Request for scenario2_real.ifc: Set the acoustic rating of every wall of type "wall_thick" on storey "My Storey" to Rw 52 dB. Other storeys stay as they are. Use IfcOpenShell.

First a look at what the model holds.

```python
import ifcopenshell
import ifcopenshell.util.element

model = ifcopenshell.open("scenario2_real.ifc")
print(model.schema)
storey = next(s for s in model.by_type("IfcBuildingStorey") if s.Name == "My Storey")
walls = [e for e in ifcopenshell.util.element.get_decomposition(storey) if e.is_a("IfcWall")]
seen = {}
for e in walls:
    element_type = ifcopenshell.util.element.get_type(e)
    key = (element_type.Name if element_type != e and element_type else None, ifcopenshell.util.element.get_pset(e, "Pset_WallCommon", "AcousticRating"))
    seen[key] = seen.get(key, 0) + 1
for (name, value), count in sorted(seen.items(), key=str):
    print(count, "x", name, "|", value)
```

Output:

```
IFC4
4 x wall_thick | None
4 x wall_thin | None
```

```python
import ifcopenshell
import ifcopenshell.api.pset
import ifcopenshell.util.element

model = ifcopenshell.open("scenario2_real.ifc")

storey = next(s for s in model.by_type("IfcBuildingStorey") if s.Name == "My Storey")
walls = [e for e in ifcopenshell.util.element.get_decomposition(storey) if e.is_a("IfcWall")]

count = 0
for e in walls:
    element_type = ifcopenshell.util.element.get_type(e)
    if element_type in (None, e) or element_type.Name != "wall_thick":
        continue
    # add_pset returns the element's existing set when there is one.
    pset = ifcopenshell.api.pset.add_pset(model, product=e, name="Pset_WallCommon")
    ifcopenshell.api.pset.edit_pset(model, pset=pset, properties={"AcousticRating": "Rw 52 dB"})
    count += 1

print(count, "walls updated")

model.write("scenario2_real_v2.ifc")
```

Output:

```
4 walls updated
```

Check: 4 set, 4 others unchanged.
